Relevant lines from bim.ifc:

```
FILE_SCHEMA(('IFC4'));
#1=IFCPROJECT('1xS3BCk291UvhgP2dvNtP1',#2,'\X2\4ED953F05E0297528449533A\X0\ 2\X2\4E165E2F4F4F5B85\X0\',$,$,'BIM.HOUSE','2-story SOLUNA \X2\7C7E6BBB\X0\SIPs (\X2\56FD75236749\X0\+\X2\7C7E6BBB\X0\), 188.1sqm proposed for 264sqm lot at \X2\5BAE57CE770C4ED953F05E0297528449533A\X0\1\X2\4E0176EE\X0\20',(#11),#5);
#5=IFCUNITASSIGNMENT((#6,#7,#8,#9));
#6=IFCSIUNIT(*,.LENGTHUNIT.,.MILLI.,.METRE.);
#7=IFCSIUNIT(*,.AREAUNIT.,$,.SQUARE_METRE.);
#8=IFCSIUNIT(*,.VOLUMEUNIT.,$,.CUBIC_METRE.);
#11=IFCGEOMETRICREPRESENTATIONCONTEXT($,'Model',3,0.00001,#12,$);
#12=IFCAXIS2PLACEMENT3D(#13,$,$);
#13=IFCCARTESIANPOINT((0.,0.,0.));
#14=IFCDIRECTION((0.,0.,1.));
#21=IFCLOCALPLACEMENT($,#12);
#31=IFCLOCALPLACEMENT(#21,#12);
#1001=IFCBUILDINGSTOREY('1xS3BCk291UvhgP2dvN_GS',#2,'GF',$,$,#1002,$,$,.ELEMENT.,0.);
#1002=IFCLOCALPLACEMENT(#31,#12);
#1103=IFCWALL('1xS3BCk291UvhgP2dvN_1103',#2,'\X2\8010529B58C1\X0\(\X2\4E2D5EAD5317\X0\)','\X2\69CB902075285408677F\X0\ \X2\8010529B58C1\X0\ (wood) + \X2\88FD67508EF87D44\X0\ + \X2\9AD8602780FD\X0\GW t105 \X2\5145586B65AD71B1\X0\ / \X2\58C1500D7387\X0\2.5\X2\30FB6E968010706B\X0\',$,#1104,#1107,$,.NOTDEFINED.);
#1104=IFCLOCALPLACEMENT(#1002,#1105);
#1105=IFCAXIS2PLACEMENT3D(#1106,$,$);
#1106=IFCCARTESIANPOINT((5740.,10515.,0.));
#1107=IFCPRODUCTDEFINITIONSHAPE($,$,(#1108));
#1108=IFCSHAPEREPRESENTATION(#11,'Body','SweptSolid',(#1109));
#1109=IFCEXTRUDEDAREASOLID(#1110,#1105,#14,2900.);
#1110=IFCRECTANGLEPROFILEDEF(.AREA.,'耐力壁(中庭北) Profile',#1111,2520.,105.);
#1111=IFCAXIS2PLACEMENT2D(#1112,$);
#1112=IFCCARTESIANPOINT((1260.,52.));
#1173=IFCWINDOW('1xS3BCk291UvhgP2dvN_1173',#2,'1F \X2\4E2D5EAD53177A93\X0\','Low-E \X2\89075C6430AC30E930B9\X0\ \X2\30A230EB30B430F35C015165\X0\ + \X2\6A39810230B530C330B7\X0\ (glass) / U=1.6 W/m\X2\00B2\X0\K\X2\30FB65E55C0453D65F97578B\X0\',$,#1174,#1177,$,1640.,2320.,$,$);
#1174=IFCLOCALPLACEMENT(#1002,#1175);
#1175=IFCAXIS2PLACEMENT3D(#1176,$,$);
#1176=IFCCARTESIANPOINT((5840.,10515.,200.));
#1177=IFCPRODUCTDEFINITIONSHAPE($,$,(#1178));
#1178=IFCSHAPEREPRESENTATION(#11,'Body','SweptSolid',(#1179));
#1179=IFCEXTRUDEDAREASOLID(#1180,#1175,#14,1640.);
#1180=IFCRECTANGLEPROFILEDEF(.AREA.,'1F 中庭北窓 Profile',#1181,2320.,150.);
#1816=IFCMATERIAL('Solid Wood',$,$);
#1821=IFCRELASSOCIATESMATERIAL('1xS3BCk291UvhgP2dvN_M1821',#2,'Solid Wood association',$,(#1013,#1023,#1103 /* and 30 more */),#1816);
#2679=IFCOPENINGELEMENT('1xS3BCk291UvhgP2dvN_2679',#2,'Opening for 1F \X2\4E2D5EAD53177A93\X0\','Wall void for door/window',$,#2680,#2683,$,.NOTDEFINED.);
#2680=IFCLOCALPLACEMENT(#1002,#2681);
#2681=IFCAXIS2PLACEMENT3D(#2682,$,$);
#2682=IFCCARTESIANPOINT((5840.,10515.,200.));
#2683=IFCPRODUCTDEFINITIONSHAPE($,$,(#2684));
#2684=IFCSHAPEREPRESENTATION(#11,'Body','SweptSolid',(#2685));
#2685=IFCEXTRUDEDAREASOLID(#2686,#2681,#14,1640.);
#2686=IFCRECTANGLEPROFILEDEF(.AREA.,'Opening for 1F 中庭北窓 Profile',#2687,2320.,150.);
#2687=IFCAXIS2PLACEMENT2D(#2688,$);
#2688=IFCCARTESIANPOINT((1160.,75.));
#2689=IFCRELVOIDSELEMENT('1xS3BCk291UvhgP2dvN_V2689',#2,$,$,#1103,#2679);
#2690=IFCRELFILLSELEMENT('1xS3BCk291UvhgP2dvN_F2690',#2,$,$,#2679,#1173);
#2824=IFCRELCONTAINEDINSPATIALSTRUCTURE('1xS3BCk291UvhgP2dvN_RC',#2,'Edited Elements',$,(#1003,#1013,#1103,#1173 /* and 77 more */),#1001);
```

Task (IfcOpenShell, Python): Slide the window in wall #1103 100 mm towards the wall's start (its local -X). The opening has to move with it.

```python
import ifcopenshell
import ifcopenshell.api.geometry
import ifcopenshell.util.placement

model = ifcopenshell.open("bim.ifc")

window = model.by_guid("1xS3BCk291UvhgP2dvN_1173")
opening = window.FillsVoids[0].RelatingOpeningElement
wall = opening.VoidsElements[0].RelatingBuildingElement

wall_matrix = ifcopenshell.util.placement.get_local_placement(wall.ObjectPlacement)
shift = wall_matrix[:3, 0] * -100.0
before = ifcopenshell.util.placement.get_local_placement(window.ObjectPlacement)[:3, 3].copy()

# The window is not placed relative to its opening, so move both.
for product in (opening, window):
    matrix = ifcopenshell.util.placement.get_local_placement(product.ObjectPlacement)
    matrix[:3, 3] += shift
    ifcopenshell.api.geometry.edit_object_placement(model, product=product, matrix=matrix, is_si=False)

after = ifcopenshell.util.placement.get_local_placement(window.ObjectPlacement)[:3, 3]
print("window moved by", (after - before).round(3) + 0.0)

model.write("bim_v2.ifc")
```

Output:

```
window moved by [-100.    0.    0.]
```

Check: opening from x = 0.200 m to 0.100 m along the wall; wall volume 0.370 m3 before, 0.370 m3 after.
